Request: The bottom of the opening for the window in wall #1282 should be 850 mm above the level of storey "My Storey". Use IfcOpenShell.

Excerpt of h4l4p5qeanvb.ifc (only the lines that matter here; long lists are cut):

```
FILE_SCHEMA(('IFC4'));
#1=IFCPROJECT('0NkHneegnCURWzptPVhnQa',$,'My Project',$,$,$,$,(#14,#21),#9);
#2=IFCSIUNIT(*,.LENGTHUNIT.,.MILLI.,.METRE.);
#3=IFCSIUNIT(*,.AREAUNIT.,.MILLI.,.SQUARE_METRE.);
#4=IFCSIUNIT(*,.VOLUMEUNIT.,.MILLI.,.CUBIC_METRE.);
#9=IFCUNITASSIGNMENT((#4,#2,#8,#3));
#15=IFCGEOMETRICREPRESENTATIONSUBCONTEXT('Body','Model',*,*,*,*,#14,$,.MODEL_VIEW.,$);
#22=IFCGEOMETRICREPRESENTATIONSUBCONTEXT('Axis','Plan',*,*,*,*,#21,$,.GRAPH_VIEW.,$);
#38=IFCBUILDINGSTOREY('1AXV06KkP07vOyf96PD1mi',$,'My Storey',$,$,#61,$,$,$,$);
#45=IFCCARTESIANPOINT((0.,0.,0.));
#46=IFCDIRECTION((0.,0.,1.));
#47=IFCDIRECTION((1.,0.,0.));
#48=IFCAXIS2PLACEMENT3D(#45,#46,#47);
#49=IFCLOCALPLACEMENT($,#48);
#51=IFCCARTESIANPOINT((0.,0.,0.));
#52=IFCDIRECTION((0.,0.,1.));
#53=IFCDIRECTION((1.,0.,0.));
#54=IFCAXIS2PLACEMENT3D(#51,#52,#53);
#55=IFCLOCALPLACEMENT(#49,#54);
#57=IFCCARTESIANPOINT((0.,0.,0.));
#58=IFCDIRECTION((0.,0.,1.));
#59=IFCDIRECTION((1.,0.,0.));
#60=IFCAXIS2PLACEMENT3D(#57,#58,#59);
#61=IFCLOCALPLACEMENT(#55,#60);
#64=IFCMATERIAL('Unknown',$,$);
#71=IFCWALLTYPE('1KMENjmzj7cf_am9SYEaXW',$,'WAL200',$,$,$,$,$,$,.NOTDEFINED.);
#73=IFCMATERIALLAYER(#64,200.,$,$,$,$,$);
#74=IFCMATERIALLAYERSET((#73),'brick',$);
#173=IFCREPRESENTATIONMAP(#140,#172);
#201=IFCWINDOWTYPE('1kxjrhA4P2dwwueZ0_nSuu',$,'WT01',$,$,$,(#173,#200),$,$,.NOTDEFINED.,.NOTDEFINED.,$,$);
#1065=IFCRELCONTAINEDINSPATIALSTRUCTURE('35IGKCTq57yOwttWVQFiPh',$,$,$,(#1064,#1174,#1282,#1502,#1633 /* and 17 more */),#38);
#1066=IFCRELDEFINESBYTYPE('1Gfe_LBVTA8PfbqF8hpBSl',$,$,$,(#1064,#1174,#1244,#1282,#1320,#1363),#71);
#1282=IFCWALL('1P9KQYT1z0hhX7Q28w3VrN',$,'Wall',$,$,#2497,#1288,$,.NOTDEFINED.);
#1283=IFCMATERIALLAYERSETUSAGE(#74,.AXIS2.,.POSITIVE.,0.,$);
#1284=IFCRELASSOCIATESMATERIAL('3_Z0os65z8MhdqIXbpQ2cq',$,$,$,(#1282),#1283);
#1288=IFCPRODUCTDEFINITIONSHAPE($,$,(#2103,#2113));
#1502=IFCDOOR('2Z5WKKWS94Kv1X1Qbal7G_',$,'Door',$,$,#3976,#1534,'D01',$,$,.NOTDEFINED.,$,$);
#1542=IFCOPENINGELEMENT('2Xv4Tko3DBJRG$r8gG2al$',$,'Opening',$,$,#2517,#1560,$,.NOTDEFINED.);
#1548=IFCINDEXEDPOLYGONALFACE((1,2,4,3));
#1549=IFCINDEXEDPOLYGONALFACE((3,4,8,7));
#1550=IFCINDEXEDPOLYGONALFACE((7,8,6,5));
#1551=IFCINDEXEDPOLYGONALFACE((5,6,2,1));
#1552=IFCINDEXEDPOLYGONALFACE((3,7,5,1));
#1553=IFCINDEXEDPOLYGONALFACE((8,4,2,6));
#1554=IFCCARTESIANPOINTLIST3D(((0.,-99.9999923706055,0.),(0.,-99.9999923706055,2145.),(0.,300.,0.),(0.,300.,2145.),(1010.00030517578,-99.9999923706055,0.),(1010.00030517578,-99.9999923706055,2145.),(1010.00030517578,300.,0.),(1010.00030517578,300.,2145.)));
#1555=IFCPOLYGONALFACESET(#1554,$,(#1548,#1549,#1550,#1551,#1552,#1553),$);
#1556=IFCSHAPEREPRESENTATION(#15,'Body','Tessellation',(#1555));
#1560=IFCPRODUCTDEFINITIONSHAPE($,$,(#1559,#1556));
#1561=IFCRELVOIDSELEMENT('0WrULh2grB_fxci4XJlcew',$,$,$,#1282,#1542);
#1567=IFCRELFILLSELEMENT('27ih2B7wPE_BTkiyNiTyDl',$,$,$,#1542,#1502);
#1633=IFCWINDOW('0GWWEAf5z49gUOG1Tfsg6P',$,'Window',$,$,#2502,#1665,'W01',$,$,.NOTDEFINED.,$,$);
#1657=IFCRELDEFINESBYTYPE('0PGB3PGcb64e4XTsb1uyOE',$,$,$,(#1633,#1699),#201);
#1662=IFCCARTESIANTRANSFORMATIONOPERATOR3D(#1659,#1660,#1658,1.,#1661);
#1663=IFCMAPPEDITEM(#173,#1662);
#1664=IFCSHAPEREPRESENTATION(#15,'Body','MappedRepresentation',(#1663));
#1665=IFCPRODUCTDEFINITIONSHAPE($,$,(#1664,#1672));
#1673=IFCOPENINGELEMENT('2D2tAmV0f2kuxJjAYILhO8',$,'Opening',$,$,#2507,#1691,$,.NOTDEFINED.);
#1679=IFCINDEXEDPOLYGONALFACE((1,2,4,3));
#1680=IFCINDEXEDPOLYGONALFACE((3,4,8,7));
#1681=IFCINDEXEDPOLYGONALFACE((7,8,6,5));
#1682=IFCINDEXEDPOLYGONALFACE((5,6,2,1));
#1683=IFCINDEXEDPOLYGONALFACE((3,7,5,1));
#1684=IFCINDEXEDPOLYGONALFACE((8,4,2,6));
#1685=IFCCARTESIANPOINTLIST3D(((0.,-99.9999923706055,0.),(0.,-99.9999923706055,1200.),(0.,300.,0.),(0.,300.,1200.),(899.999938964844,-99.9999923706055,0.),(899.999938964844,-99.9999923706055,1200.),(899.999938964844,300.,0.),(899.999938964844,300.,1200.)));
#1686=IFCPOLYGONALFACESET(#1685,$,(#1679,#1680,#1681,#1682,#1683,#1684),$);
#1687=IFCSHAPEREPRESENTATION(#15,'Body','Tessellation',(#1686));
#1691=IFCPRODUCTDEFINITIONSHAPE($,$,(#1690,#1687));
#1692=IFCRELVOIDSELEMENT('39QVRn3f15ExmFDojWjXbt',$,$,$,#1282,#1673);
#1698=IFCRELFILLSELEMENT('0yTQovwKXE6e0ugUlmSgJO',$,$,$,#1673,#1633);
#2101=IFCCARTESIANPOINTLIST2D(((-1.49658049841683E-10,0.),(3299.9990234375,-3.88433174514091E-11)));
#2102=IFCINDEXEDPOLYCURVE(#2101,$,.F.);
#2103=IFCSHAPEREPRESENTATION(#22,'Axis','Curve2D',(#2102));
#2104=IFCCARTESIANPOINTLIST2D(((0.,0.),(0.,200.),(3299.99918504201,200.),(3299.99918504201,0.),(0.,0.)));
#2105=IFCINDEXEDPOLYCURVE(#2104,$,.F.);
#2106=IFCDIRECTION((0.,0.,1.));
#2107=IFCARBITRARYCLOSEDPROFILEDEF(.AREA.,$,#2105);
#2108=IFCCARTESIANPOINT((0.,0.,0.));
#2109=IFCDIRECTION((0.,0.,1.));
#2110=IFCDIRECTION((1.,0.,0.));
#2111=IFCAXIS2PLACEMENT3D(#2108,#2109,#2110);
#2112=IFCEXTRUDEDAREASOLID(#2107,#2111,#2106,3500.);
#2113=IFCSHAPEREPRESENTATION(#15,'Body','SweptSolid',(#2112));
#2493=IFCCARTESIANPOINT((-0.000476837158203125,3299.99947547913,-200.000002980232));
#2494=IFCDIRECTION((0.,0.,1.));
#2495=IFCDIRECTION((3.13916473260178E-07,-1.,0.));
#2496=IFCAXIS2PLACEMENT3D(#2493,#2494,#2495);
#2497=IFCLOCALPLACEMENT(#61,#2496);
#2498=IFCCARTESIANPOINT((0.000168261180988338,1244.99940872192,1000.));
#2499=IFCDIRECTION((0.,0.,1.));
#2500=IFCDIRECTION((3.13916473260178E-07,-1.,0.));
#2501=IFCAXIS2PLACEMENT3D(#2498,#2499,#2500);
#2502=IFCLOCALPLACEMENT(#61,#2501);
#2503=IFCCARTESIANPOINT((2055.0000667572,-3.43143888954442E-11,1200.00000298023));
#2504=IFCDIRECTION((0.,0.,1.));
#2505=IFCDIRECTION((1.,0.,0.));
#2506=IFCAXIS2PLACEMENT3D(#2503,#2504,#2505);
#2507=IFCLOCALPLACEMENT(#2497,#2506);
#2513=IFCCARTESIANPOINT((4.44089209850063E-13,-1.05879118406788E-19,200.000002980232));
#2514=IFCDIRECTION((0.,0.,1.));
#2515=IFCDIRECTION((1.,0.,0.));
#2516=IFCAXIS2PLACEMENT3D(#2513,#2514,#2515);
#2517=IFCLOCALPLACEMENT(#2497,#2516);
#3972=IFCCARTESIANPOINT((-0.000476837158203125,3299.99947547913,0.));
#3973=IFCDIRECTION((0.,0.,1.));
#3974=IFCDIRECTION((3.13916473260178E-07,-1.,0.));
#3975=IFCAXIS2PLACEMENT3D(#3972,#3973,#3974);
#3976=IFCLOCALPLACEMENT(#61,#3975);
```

```python
import numpy as np
import ifcopenshell
import ifcopenshell.api.geometry
import ifcopenshell.geom
import ifcopenshell.util.element
import ifcopenshell.util.placement
import ifcopenshell.util.shape
import ifcopenshell.util.unit

model = ifcopenshell.open("h4l4p5qeanvb.ifc")
unit_scale = ifcopenshell.util.unit.calculate_unit_scale(model)

window = model.by_id(1633)
opening = window.FillsVoids[0].RelatingOpeningElement
storey = ifcopenshell.util.element.get_container(window, ifc_class="IfcBuildingStorey")
level = ifcopenshell.util.placement.get_local_placement(storey.ObjectPlacement)[2, 3]

# The opening's origin need not be at the sill, so measure its lowest point.
shape = ifcopenshell.geom.create_shape(ifcopenshell.geom.settings(), opening)
bottom = ifcopenshell.util.shape.get_shape_bottom_elevation(shape, shape.geometry) / unit_scale
dz = level + 0.85 / unit_scale - bottom

shift = np.array([0.0, 0.0, dz])
# The window is not placed relative to its opening, so move both.
for product in (opening, window):
    matrix = ifcopenshell.util.placement.get_local_placement(product.ObjectPlacement)
    matrix[:3, 3] += shift
    ifcopenshell.api.geometry.edit_object_placement(model, product=product, matrix=matrix, is_si=False)

print(f"moved by {dz * unit_scale:+.3f} m")

model.write("h4l4p5qeanvb-out.ifc")
```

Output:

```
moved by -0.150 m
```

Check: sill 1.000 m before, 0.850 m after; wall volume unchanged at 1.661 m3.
